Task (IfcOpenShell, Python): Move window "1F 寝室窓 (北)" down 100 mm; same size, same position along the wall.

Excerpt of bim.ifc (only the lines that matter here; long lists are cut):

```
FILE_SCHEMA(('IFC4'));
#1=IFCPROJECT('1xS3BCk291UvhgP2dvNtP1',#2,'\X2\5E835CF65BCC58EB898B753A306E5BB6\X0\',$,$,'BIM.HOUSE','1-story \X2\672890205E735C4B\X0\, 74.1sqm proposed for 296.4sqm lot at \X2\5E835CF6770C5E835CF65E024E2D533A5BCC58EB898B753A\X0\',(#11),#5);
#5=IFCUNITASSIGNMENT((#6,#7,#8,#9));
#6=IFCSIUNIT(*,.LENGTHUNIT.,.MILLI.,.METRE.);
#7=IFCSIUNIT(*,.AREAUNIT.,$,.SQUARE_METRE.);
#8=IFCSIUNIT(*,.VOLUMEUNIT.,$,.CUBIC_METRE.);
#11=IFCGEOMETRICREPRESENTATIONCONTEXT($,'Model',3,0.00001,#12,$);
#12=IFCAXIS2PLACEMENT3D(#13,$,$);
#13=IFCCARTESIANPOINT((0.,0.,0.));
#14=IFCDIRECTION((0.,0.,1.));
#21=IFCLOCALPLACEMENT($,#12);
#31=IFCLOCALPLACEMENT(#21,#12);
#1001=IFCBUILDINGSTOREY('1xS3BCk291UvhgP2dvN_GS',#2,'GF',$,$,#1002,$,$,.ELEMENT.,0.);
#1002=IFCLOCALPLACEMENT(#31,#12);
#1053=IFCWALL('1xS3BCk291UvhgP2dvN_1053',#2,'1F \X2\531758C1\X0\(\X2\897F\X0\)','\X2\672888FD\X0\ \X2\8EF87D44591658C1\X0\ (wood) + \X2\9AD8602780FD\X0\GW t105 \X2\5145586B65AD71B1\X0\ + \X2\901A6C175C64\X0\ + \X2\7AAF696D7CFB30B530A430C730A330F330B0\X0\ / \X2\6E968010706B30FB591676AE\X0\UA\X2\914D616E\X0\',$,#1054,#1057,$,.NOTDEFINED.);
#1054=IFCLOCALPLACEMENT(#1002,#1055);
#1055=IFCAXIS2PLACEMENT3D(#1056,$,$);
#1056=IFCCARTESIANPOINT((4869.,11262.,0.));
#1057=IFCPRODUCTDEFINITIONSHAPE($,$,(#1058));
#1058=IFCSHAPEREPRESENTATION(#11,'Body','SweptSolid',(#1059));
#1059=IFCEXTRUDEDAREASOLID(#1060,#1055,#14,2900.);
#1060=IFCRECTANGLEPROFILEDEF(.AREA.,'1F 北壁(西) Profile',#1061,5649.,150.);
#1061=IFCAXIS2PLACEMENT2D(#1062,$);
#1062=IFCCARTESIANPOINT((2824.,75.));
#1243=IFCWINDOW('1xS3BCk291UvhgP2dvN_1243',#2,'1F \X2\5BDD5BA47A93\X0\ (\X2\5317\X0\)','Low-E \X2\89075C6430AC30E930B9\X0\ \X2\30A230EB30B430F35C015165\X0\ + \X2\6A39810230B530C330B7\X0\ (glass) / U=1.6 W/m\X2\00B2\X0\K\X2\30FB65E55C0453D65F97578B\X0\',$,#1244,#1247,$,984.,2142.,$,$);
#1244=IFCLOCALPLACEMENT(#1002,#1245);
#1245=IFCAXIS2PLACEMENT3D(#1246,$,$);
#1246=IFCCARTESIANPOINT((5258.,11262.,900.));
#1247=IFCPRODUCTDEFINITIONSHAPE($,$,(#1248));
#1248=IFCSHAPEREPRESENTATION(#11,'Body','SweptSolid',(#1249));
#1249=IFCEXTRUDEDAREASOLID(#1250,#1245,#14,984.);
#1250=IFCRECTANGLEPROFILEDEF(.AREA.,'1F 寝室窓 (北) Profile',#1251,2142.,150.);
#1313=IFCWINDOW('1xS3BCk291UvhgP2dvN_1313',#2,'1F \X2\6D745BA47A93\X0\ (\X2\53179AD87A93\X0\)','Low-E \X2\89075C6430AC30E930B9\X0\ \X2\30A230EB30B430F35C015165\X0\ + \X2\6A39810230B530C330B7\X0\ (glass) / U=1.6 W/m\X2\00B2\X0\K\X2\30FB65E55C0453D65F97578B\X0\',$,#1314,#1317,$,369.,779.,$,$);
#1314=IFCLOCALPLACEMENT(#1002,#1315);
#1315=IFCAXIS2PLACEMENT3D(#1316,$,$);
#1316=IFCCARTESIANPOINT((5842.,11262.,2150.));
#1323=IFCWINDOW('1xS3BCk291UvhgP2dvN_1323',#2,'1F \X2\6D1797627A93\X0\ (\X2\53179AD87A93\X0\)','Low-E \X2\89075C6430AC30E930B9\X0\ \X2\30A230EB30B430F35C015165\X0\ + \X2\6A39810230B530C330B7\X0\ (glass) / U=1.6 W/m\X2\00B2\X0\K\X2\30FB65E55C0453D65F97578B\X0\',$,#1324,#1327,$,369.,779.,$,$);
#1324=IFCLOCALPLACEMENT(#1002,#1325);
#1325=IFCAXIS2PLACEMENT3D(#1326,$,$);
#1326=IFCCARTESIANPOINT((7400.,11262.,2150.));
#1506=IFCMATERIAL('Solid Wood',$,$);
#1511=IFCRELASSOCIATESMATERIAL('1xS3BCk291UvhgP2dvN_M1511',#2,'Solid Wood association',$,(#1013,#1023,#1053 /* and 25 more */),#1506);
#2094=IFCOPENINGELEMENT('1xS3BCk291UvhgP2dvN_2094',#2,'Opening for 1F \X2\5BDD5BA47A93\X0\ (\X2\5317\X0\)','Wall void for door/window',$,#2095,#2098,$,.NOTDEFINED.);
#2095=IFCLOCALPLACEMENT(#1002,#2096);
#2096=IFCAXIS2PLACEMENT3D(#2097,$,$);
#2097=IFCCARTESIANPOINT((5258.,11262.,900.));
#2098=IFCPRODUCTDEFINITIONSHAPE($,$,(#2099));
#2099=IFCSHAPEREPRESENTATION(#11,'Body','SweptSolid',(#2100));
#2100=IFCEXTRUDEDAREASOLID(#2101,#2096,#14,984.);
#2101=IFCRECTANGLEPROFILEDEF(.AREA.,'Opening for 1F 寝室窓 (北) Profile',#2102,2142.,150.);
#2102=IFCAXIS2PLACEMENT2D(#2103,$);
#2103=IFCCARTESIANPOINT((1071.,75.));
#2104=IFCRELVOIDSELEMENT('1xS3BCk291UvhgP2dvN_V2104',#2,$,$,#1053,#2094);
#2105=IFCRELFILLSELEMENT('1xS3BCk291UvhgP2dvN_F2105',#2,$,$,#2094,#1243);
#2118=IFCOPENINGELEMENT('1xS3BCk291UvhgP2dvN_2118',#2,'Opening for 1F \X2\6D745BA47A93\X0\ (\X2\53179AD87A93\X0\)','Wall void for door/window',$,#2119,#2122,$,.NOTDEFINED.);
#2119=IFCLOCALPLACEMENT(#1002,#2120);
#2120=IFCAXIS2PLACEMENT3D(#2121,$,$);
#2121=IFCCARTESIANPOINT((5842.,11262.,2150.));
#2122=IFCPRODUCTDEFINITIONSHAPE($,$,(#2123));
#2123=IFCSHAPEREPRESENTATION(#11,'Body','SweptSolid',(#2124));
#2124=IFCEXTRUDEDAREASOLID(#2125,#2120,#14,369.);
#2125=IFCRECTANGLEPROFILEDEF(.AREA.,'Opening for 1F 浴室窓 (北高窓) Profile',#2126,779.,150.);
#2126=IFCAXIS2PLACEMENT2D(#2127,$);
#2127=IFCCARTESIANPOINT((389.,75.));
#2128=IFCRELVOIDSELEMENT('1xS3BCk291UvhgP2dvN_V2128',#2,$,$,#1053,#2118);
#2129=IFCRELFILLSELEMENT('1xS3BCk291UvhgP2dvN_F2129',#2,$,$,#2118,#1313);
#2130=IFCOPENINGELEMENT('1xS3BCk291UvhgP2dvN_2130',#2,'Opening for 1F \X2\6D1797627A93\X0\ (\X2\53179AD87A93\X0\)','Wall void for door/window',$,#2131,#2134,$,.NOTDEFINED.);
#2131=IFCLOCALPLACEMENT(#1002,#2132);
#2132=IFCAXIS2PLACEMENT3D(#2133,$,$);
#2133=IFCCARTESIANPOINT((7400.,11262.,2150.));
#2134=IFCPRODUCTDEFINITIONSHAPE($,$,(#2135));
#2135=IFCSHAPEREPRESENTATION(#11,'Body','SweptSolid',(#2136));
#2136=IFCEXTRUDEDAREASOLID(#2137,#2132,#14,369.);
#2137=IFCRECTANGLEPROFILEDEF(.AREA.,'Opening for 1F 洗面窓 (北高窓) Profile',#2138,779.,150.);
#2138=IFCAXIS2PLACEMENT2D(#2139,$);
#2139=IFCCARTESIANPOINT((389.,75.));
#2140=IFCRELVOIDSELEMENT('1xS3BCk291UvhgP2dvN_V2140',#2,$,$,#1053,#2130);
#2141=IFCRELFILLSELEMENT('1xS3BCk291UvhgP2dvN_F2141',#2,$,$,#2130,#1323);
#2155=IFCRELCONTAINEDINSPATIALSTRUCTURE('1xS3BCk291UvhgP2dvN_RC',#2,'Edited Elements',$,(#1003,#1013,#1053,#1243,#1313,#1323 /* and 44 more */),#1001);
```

```python
import numpy as np
import ifcopenshell
import ifcopenshell.api.geometry
import ifcopenshell.util.placement
import ifcopenshell.util.unit

model = ifcopenshell.open("bim.ifc")
unit_scale = ifcopenshell.util.unit.calculate_unit_scale(model)

window = model.by_guid("1xS3BCk291UvhgP2dvN_1243")
opening = window.FillsVoids[0].RelatingOpeningElement
dz = -100.0

shift = np.array([0.0, 0.0, dz])
# The window is not placed relative to its opening, so move both.
for product in (opening, window):
    matrix = ifcopenshell.util.placement.get_local_placement(product.ObjectPlacement)
    matrix[:3, 3] += shift
    ifcopenshell.api.geometry.edit_object_placement(model, product=product, matrix=matrix, is_si=False)

print(f"moved by {dz * unit_scale:+.3f} m")

model.write("bim_v2.ifc")
```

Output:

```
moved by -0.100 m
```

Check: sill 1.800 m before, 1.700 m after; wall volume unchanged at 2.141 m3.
